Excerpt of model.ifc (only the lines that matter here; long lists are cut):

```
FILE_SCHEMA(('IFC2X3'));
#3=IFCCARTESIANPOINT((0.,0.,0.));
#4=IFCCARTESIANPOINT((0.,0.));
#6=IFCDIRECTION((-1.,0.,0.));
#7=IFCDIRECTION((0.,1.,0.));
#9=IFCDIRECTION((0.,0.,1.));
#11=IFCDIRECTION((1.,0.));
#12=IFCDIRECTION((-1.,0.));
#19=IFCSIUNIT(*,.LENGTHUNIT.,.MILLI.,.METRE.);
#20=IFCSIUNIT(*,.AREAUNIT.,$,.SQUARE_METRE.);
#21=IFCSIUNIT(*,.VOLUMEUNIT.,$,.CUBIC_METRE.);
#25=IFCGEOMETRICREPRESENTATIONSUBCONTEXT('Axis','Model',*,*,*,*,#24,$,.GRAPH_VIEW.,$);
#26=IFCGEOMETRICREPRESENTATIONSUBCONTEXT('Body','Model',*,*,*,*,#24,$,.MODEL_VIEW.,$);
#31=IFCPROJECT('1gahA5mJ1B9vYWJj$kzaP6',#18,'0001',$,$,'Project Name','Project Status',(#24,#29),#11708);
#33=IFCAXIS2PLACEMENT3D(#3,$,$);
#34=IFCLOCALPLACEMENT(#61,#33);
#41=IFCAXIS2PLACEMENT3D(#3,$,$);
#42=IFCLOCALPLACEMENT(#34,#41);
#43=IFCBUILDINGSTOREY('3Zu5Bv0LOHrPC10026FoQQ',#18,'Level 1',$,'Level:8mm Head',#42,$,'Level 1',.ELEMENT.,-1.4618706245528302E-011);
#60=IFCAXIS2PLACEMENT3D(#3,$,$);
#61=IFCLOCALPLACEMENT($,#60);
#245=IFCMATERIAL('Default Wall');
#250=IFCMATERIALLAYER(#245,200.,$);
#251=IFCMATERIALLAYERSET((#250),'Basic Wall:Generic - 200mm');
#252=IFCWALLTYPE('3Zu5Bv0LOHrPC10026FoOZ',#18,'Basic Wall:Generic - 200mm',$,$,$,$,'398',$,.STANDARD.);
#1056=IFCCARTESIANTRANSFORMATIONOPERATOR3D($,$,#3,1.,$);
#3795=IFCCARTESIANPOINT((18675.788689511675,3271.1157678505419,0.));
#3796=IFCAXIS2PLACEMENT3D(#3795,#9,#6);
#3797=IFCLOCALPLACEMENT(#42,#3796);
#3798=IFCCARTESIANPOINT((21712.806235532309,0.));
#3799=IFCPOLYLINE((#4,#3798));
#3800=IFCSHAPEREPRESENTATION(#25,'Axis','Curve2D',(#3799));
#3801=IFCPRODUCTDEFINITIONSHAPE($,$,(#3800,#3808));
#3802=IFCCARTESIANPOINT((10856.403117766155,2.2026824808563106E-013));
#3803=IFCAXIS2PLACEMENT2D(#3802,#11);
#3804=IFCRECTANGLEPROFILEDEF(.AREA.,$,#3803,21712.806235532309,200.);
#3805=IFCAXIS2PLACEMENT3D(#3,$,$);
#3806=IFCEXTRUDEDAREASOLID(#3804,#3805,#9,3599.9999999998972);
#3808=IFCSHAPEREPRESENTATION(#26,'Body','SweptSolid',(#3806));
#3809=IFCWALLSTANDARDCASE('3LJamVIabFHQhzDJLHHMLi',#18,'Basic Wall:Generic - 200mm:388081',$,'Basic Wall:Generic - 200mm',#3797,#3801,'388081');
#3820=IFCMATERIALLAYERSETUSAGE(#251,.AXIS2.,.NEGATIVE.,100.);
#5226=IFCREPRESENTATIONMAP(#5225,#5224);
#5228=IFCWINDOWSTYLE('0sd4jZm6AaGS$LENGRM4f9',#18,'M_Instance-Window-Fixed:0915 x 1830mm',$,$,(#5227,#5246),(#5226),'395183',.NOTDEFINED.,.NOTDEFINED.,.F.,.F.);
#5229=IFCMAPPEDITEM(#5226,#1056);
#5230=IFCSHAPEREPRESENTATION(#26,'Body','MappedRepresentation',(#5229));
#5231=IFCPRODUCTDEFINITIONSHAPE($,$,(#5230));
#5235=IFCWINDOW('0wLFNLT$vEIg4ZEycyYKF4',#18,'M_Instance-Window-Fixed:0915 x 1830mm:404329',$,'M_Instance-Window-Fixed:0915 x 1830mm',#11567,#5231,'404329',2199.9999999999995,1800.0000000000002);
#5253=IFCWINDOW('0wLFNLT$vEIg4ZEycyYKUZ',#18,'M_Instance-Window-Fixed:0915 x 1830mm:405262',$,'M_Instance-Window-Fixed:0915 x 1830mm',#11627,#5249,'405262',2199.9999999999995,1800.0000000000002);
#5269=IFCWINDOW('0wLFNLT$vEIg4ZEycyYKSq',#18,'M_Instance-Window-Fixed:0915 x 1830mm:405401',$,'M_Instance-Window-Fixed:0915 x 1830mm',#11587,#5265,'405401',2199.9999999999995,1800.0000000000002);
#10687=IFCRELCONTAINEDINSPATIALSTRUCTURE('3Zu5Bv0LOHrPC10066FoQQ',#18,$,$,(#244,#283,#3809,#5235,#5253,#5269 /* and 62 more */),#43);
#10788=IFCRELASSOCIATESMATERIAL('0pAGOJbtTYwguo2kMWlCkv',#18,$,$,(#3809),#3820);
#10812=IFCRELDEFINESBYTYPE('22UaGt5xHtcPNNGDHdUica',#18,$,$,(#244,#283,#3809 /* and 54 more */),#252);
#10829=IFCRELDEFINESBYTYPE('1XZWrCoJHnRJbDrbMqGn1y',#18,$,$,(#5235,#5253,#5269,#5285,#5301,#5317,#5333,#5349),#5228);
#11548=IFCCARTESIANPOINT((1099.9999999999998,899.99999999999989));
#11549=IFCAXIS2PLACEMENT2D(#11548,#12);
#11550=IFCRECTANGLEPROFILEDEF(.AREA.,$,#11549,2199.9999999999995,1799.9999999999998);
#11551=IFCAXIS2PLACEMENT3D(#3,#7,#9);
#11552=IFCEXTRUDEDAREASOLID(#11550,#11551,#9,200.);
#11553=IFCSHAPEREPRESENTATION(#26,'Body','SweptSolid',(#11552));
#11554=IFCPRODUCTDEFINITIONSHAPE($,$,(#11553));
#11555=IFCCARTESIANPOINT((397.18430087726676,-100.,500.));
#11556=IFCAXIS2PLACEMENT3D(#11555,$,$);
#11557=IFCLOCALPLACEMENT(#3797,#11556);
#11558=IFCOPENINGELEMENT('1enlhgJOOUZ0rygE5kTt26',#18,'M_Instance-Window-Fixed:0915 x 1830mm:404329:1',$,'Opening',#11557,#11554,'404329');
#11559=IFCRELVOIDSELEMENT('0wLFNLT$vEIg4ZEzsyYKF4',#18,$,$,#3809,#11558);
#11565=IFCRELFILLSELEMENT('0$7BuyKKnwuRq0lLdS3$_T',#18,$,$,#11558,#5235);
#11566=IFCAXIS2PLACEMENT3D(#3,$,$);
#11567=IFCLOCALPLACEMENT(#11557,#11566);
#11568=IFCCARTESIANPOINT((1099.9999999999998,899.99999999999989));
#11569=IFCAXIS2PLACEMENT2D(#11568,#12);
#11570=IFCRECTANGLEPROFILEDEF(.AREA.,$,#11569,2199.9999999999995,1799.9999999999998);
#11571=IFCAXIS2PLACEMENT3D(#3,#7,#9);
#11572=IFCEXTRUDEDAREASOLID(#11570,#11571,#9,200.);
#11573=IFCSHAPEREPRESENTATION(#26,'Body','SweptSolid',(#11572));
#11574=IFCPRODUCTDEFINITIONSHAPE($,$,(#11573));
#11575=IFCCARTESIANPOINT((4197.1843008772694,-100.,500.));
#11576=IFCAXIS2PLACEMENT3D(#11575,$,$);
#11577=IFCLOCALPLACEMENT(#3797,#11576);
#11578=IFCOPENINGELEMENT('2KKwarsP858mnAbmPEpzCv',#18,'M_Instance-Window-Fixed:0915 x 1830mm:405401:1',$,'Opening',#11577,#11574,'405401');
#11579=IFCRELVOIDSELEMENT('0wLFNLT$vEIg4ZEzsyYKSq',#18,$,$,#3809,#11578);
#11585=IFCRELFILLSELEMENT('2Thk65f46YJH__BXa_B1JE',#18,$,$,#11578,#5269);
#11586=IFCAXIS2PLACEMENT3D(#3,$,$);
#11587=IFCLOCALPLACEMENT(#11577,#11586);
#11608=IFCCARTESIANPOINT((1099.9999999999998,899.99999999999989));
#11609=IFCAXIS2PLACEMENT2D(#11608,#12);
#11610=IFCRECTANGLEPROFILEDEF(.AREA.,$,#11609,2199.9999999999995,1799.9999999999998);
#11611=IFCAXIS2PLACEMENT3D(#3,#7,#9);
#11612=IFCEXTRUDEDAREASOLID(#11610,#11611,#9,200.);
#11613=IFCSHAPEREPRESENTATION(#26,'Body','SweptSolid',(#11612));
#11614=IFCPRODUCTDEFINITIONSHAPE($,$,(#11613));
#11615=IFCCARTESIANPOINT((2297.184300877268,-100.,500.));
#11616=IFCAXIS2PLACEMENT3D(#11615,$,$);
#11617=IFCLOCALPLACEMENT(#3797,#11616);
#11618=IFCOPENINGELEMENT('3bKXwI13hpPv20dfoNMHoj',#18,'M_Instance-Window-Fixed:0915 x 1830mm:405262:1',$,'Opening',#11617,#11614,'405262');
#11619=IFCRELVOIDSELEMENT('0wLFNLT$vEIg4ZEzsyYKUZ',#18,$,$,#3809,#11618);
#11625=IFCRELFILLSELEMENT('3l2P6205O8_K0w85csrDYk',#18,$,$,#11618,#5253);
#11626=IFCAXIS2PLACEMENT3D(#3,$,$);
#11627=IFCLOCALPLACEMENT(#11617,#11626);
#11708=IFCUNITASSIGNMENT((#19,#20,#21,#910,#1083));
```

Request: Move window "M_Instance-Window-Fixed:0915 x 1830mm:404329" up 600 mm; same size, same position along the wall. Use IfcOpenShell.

```python
import numpy as np
import ifcopenshell
import ifcopenshell.api.geometry
import ifcopenshell.util.placement
import ifcopenshell.util.unit

model = ifcopenshell.open("model.ifc")
unit_scale = ifcopenshell.util.unit.calculate_unit_scale(model)

window = model.by_guid("0wLFNLT$vEIg4ZEycyYKF4")
opening = window.FillsVoids[0].RelatingOpeningElement
dz = 600.0

shift = np.array([0.0, 0.0, dz])
# The window is placed relative to its opening, so it follows when the opening moves.
matrix = ifcopenshell.util.placement.get_local_placement(opening.ObjectPlacement)
matrix[:3, 3] += shift
ifcopenshell.api.geometry.edit_object_placement(
    model, product=opening, matrix=matrix, is_si=False, should_transform_children=True
)

print(f"moved by {dz * unit_scale:+.3f} m")

model.write("model_edited.ifc")
```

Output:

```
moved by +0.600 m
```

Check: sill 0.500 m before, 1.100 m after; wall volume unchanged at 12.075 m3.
